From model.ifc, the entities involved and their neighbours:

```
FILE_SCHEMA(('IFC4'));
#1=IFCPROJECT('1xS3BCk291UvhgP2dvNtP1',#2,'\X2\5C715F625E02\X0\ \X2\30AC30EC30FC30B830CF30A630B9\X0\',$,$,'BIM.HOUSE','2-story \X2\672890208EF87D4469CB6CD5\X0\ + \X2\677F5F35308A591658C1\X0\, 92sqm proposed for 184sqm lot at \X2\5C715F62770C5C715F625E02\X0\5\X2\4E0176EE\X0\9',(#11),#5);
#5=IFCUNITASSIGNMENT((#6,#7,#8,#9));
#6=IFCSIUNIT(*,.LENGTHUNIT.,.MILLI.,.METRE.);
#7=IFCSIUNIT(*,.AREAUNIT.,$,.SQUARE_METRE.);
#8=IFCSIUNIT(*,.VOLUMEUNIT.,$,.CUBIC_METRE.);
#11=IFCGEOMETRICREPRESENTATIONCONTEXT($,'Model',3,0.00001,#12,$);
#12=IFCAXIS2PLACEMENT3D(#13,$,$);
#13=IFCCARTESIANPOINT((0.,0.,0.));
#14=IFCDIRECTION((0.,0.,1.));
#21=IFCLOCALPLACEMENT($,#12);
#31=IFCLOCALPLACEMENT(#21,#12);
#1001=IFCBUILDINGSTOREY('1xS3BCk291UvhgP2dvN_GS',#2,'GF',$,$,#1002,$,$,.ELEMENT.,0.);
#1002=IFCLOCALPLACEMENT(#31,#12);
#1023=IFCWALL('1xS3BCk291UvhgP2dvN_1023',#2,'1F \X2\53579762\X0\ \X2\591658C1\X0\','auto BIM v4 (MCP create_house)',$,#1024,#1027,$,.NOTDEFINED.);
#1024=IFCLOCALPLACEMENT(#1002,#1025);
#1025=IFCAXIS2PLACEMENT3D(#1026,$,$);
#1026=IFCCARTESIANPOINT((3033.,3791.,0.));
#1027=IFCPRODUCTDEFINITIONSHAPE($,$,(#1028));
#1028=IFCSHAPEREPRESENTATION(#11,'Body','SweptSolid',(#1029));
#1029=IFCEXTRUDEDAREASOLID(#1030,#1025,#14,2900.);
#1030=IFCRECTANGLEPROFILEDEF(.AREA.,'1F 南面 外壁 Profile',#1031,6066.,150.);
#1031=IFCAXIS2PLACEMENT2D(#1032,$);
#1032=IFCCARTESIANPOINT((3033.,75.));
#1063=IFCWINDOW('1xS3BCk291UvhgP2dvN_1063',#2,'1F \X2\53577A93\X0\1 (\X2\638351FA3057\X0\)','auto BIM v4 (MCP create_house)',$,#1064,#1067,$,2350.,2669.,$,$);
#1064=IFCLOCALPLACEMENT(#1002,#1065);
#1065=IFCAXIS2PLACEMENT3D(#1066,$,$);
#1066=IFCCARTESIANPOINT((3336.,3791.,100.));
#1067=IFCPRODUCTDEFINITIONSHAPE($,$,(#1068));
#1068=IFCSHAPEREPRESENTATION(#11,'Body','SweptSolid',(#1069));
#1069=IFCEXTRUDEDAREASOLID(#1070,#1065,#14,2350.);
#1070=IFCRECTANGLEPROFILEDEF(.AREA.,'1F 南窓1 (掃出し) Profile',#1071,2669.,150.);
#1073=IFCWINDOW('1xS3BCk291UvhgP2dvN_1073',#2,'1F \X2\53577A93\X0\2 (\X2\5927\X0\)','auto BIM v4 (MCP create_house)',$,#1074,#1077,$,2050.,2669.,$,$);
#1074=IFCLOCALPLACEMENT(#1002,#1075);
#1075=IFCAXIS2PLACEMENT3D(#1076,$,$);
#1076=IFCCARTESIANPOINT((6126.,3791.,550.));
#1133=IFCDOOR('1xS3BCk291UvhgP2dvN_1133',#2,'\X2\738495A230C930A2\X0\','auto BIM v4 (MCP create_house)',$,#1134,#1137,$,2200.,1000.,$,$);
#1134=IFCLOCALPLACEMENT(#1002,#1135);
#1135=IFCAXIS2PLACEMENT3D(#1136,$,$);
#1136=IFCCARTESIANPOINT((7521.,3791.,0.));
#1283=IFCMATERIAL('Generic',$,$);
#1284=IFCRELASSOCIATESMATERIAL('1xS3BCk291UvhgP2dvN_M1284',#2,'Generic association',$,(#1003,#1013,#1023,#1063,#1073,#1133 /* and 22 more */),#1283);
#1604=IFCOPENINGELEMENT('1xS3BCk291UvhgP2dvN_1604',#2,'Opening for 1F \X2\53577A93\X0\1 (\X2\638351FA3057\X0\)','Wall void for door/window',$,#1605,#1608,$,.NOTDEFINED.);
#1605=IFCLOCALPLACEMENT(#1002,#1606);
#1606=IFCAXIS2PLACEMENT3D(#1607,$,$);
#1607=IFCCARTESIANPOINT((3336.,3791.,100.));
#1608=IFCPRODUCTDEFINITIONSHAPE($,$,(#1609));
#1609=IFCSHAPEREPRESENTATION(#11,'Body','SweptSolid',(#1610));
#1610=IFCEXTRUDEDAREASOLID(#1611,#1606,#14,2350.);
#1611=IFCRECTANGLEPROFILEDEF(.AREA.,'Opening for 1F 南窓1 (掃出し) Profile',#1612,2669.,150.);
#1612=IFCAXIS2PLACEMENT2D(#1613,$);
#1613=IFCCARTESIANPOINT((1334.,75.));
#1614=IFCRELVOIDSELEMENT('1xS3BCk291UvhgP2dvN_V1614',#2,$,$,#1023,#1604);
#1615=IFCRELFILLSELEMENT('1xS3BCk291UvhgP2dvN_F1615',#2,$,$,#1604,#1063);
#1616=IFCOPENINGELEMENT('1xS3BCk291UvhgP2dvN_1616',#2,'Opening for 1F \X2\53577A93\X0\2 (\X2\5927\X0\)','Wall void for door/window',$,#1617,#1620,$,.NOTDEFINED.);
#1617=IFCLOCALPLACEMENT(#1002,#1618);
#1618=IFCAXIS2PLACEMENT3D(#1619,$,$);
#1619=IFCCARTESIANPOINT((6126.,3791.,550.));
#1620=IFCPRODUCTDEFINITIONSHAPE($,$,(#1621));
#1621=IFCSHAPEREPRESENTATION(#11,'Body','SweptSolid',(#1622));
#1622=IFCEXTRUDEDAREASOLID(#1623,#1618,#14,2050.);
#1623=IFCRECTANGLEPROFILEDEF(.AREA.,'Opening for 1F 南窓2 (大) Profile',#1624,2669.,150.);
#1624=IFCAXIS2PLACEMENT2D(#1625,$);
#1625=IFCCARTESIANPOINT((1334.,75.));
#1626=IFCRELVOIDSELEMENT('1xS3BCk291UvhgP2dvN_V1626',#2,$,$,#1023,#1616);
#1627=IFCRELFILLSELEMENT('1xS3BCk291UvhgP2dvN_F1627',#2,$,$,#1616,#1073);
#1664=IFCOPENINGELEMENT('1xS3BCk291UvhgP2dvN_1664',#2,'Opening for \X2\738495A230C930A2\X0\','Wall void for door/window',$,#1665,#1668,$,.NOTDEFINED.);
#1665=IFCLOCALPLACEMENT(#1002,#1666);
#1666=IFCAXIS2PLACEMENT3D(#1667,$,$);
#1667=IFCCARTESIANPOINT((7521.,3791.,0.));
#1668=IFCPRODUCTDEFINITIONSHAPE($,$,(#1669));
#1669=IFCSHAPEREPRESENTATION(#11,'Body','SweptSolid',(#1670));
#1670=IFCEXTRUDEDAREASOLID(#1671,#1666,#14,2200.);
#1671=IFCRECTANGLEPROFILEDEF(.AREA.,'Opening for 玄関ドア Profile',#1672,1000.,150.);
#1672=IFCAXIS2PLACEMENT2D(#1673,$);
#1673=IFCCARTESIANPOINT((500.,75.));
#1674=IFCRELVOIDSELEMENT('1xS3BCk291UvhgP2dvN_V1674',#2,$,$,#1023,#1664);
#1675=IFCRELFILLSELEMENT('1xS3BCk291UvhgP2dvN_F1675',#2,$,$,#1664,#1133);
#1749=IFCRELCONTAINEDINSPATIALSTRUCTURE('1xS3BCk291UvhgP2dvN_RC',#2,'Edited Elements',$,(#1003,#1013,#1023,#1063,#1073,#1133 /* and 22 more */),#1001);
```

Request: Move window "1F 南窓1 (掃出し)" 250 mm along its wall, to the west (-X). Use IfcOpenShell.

```python
import ifcopenshell
import ifcopenshell.api.geometry
import ifcopenshell.util.placement

model = ifcopenshell.open("model.ifc")

window = model.by_id(1063)
opening = window.FillsVoids[0].RelatingOpeningElement
wall = opening.VoidsElements[0].RelatingBuildingElement

wall_matrix = ifcopenshell.util.placement.get_local_placement(wall.ObjectPlacement)
shift = wall_matrix[:3, 0] * -250.0
before = ifcopenshell.util.placement.get_local_placement(window.ObjectPlacement)[:3, 3].copy()

# The window is not placed relative to its opening, so move both.
for product in (opening, window):
    matrix = ifcopenshell.util.placement.get_local_placement(product.ObjectPlacement)
    matrix[:3, 3] += shift
    ifcopenshell.api.geometry.edit_object_placement(model, product=product, matrix=matrix, is_si=False)

after = ifcopenshell.util.placement.get_local_placement(window.ObjectPlacement)[:3, 3]
print("window moved by", (after - before).round(3) + 0.0)

model.write("model_updated.ifc")
```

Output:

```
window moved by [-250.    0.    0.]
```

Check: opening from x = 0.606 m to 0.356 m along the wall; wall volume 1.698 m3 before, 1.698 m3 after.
